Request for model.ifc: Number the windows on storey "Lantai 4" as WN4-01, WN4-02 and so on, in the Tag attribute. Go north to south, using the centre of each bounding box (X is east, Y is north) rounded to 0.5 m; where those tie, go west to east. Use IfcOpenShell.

First a look at what the model holds.

```python
import ifcopenshell
import ifcopenshell.util.element
import ifcopenshell.util.placement

model = ifcopenshell.open("model.ifc")
print(model.schema)
storey = next(s for s in model.by_type("IfcBuildingStorey") if s.Name == "Lantai 4")
windows = [e for e in ifcopenshell.util.element.get_decomposition(storey) if e.is_a("IfcWindow")]
for e in sorted(windows, key=lambda e: e.id()):
    origin = ifcopenshell.util.placement.get_local_placement(e.ObjectPlacement)[:3, 3]
    print(e.id(), e.Tag, e.Name, origin.round(2) + 0.0, sep=" | ")
```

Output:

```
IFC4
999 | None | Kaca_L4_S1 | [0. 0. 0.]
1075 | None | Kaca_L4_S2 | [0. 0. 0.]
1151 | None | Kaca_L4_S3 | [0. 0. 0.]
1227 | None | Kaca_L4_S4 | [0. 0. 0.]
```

```python
import ifcopenshell
import ifcopenshell.geom
import ifcopenshell.util.element
import ifcopenshell.util.shape

model = ifcopenshell.open("model.ifc")
settings = ifcopenshell.geom.settings()
settings.set("use-world-coords", True)


def centre(element):
    shape = ifcopenshell.geom.create_shape(settings, element)
    return ifcopenshell.util.shape.get_bbox_centroid(shape.geometry)


storey = next(s for s in model.by_type("IfcBuildingStorey") if s.Name == "Lantai 4")
windows = [e for e in ifcopenshell.util.element.get_decomposition(storey) if e.is_a("IfcWindow")]

# Insertion points can sit at a corner or the storey origin, so sort by the geometry (in metres).
centres = {e: centre(e) for e in windows}
windows.sort(key=lambda e: (-round(centres[e][1] / 0.5), centres[e][0]))

for i, e in enumerate(windows, start=1):
    number = f"WN4-{i:02d}"
    e.Tag = number
    print(e.id(), number)

model.write("model_edited.ifc")
```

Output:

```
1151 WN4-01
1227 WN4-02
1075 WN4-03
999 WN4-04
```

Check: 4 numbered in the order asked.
